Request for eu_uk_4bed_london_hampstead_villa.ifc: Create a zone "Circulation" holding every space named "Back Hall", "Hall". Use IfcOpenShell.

First a look at what the model holds.

```python
import ifcopenshell

model = ifcopenshell.open("eu_uk_4bed_london_hampstead_villa.ifc")
print(model.schema)
seen = {}
for space in model.by_type("IfcSpace"):
    seen[space.LongName] = seen.get(space.LongName, 0) + 1
for name, count in sorted(seen.items(), key=str):
    print(count, "x", name)
print("zones:", [z.Name for z in model.by_type("IfcZone")][:20])
```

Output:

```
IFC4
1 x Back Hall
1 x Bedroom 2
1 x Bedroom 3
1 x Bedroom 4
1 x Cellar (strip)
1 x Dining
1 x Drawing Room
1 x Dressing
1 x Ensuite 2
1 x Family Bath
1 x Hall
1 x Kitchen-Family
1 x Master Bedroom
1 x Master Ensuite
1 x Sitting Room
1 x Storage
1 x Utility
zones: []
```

```python
import ifcopenshell
import ifcopenshell.api.group
import ifcopenshell.api.root

model = ifcopenshell.open("eu_uk_4bed_london_hampstead_villa.ifc")

names = {"Back Hall", "Hall"}
spaces = [s for s in model.by_type("IfcSpace") if s.LongName in names]

zone = ifcopenshell.api.root.create_entity(model, ifc_class="IfcZone", name="Circulation")
ifcopenshell.api.group.assign_group(model, products=spaces, group=zone)
print(len(spaces), "spaces in", zone.Name)

model.write("eu_uk_4bed_london_hampstead_villa_rev.ifc")
```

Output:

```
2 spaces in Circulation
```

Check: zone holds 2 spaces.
